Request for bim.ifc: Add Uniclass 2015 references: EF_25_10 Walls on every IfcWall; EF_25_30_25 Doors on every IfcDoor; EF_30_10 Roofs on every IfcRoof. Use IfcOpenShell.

First a look at what the model holds.

```python
import ifcopenshell

model = ifcopenshell.open("bim.ifc")
print(model.schema)
print("classifications:", [c.Name for c in model.by_type("IfcClassification")])
for ifc_class in ("IfcDoor", "IfcRoof", "IfcStair", "IfcWall", "IfcWindow"):
    print(ifc_class, len(model.by_type(ifc_class)))
```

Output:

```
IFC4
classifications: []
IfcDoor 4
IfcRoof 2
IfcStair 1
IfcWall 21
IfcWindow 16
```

```python
import ifcopenshell
import ifcopenshell.api.classification

model = ifcopenshell.open("bim.ifc")

system = ifcopenshell.api.classification.add_classification(model, classification="Uniclass 2015")

codes = {
    "IfcWall": ("EF_25_10", "Walls"),
    "IfcDoor": ("EF_25_30_25", "Doors"),
    "IfcRoof": ("EF_30_10", "Roofs"),
}
for ifc_class, (code, name) in codes.items():
    products = model.by_type(ifc_class)
    ifcopenshell.api.classification.add_reference(
        model, products=products, classification=system, identification=code, name=name
    )
    print(code, len(products))

model.write("bim_rev.ifc")
```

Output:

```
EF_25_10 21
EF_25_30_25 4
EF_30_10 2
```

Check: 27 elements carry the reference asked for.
